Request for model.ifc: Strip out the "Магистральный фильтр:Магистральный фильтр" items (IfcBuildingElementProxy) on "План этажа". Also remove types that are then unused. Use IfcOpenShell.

First a look at what the model holds.

```python
import ifcopenshell
import ifcopenshell.util.element

model = ifcopenshell.open("model.ifc")
print(model.schema)
storey = next(s for s in model.by_type("IfcBuildingStorey") if s.Name == "План этажа")
proxies = [e for e in ifcopenshell.util.element.get_decomposition(storey) if e.is_a("IfcBuildingElementProxy")]
seen = {}
for e in proxies:
    element_type = ifcopenshell.util.element.get_type(e)
    name = element_type.Name if element_type not in (None, e) else None
    seen[name] = seen.get(name, 0) + 1
for name, count in sorted(seen.items(), key=str):
    print(count, "x", name)
```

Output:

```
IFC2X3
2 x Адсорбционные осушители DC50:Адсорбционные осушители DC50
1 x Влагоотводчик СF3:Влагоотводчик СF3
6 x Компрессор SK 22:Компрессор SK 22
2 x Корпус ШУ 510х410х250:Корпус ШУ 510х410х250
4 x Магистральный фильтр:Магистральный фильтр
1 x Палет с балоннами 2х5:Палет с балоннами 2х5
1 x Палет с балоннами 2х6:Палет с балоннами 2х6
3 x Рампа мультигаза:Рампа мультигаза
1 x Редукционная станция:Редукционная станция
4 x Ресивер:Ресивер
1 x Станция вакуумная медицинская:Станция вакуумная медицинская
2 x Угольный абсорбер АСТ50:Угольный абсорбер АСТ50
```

```python
import ifcopenshell
import ifcopenshell.api.root
import ifcopenshell.util.element

model = ifcopenshell.open("model.ifc")

storey = next(s for s in model.by_type("IfcBuildingStorey") if s.Name == "План этажа")
proxies = [e for e in ifcopenshell.util.element.get_decomposition(storey) if e.is_a("IfcBuildingElementProxy")]
targets = [e for e in proxies if (t := ifcopenshell.util.element.get_type(e)) not in (None, e) and t.Name == "Магистральный фильтр:Магистральный фильтр"]
types = {ifcopenshell.util.element.get_type(e) for e in targets} - {None, *targets}

for e in targets:
    ifcopenshell.api.root.remove_product(model, product=e)
print(len(targets), "removed")

unused = [t for t in types if not ifcopenshell.util.element.get_types(t)]
for t in unused:
    ifcopenshell.api.root.remove_product(model, product=t)
print(len(unused), "unused types removed")

model.write("model_updated.ifc")
```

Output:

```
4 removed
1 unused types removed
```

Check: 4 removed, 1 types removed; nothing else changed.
